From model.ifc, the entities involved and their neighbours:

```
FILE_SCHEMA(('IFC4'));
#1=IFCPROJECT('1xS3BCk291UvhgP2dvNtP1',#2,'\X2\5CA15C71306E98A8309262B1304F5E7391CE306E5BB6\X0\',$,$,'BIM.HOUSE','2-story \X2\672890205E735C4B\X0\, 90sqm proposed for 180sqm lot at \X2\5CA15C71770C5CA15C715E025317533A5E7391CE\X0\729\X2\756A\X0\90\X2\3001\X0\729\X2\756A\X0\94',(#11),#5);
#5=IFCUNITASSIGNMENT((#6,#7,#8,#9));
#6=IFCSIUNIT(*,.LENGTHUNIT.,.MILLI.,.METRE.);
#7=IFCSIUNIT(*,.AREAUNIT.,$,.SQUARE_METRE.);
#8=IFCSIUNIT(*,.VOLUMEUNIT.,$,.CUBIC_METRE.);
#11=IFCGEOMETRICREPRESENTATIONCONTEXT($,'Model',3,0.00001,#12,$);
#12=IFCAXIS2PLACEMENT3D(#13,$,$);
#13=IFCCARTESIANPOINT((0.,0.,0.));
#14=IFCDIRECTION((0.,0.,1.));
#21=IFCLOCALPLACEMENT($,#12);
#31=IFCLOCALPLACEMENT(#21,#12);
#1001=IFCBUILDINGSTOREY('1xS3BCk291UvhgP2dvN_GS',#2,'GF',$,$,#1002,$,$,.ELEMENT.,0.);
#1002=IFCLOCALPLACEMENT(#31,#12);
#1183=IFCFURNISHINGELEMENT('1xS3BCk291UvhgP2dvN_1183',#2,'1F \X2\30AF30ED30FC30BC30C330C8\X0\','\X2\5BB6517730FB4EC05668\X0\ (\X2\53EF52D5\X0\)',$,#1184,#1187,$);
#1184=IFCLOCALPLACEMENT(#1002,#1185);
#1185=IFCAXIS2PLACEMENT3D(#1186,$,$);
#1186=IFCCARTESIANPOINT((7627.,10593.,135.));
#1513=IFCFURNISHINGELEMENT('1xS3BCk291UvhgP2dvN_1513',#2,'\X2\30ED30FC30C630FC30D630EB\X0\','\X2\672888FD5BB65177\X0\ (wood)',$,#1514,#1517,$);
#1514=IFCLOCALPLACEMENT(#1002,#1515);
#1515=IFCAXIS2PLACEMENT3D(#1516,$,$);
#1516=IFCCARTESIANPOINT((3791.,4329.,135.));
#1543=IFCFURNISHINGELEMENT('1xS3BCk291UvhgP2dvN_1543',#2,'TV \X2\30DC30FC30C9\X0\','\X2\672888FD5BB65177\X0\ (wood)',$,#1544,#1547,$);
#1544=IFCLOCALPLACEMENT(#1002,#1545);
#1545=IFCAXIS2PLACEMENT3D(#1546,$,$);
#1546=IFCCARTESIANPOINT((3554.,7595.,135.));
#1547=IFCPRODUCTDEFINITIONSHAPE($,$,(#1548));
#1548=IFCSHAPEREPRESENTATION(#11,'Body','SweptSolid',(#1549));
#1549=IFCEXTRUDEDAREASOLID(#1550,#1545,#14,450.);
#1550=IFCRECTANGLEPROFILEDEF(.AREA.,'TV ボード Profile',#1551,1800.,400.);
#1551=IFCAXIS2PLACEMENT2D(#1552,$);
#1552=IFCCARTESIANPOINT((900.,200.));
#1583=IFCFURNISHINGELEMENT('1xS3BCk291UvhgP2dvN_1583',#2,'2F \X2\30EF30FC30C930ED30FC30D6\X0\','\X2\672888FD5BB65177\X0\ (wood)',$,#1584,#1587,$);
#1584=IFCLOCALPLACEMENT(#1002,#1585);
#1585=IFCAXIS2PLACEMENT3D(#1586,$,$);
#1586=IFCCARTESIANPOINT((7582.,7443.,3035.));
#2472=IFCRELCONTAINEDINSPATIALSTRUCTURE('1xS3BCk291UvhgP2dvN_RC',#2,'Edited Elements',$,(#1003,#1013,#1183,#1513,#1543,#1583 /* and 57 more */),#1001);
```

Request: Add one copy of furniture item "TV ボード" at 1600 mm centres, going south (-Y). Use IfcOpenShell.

```python
import numpy as np
import ifcopenshell
import ifcopenshell.api.geometry
import ifcopenshell.api.root
import ifcopenshell.util.element
import ifcopenshell.util.placement

model = ifcopenshell.open("model.ifc")


def reuse_history(source, copy):
    """copy_class also copies each property set's owner history, people and application; keep the originals."""
    for rel in copy.IsDefinedBy:
        if rel.is_a("IfcRelDefinesByProperties") and (history := rel.RelatingPropertyDefinition.OwnerHistory):
            rel.RelatingPropertyDefinition.OwnerHistory = source.OwnerHistory
            ifcopenshell.util.element.remove_deep2(model, history)


source = model.by_guid("1xS3BCk291UvhgP2dvN_1543")
base = ifcopenshell.util.placement.get_local_placement(source.ObjectPlacement)
step = np.array([0.0, -1.0, 0.0]) * 1600.0

for i in range(1, 2):
    copy = ifcopenshell.api.root.copy_class(model, product=source)
    copy.Representation = ifcopenshell.util.element.copy_deep(
        model, source.Representation, exclude=["IfcGeometricRepresentationContext", "IfcRepresentationMap"]
    )
    reuse_history(source, copy)
    matrix = base.copy()
    matrix[:3, 3] += i * step
    print("added at", matrix[:3, 3].round(3) + 0.0)
    ifcopenshell.api.geometry.edit_object_placement(model, product=copy, matrix=matrix, is_si=False)

model.write("model_edited.ifc")
```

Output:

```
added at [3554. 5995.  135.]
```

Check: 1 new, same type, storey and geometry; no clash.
